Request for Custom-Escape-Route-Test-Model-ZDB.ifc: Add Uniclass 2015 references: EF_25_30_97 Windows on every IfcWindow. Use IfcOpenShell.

First a look at what the model holds.

```python
import ifcopenshell

model = ifcopenshell.open("Custom-Escape-Route-Test-Model-ZDB.ifc")
print(model.schema)
print("classifications:", [c.Name for c in model.by_type("IfcClassification")])
for ifc_class in ("IfcDoor", "IfcRoof", "IfcStair", "IfcWall", "IfcWindow"):
    print(ifc_class, len(model.by_type(ifc_class)))
```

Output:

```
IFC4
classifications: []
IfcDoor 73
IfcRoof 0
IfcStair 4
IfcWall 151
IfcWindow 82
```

```python
import ifcopenshell
import ifcopenshell.api.classification

model = ifcopenshell.open("Custom-Escape-Route-Test-Model-ZDB.ifc")

system = ifcopenshell.api.classification.add_classification(model, classification="Uniclass 2015")

codes = {
    "IfcWindow": ("EF_25_30_97", "Windows"),
}
for ifc_class, (code, name) in codes.items():
    products = model.by_type(ifc_class)
    ifcopenshell.api.classification.add_reference(
        model, products=products, classification=system, identification=code, name=name
    )
    print(code, len(products))

model.write("Custom-Escape-Route-Test-Model-ZDB_rev.ifc")
```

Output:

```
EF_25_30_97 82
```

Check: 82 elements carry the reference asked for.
